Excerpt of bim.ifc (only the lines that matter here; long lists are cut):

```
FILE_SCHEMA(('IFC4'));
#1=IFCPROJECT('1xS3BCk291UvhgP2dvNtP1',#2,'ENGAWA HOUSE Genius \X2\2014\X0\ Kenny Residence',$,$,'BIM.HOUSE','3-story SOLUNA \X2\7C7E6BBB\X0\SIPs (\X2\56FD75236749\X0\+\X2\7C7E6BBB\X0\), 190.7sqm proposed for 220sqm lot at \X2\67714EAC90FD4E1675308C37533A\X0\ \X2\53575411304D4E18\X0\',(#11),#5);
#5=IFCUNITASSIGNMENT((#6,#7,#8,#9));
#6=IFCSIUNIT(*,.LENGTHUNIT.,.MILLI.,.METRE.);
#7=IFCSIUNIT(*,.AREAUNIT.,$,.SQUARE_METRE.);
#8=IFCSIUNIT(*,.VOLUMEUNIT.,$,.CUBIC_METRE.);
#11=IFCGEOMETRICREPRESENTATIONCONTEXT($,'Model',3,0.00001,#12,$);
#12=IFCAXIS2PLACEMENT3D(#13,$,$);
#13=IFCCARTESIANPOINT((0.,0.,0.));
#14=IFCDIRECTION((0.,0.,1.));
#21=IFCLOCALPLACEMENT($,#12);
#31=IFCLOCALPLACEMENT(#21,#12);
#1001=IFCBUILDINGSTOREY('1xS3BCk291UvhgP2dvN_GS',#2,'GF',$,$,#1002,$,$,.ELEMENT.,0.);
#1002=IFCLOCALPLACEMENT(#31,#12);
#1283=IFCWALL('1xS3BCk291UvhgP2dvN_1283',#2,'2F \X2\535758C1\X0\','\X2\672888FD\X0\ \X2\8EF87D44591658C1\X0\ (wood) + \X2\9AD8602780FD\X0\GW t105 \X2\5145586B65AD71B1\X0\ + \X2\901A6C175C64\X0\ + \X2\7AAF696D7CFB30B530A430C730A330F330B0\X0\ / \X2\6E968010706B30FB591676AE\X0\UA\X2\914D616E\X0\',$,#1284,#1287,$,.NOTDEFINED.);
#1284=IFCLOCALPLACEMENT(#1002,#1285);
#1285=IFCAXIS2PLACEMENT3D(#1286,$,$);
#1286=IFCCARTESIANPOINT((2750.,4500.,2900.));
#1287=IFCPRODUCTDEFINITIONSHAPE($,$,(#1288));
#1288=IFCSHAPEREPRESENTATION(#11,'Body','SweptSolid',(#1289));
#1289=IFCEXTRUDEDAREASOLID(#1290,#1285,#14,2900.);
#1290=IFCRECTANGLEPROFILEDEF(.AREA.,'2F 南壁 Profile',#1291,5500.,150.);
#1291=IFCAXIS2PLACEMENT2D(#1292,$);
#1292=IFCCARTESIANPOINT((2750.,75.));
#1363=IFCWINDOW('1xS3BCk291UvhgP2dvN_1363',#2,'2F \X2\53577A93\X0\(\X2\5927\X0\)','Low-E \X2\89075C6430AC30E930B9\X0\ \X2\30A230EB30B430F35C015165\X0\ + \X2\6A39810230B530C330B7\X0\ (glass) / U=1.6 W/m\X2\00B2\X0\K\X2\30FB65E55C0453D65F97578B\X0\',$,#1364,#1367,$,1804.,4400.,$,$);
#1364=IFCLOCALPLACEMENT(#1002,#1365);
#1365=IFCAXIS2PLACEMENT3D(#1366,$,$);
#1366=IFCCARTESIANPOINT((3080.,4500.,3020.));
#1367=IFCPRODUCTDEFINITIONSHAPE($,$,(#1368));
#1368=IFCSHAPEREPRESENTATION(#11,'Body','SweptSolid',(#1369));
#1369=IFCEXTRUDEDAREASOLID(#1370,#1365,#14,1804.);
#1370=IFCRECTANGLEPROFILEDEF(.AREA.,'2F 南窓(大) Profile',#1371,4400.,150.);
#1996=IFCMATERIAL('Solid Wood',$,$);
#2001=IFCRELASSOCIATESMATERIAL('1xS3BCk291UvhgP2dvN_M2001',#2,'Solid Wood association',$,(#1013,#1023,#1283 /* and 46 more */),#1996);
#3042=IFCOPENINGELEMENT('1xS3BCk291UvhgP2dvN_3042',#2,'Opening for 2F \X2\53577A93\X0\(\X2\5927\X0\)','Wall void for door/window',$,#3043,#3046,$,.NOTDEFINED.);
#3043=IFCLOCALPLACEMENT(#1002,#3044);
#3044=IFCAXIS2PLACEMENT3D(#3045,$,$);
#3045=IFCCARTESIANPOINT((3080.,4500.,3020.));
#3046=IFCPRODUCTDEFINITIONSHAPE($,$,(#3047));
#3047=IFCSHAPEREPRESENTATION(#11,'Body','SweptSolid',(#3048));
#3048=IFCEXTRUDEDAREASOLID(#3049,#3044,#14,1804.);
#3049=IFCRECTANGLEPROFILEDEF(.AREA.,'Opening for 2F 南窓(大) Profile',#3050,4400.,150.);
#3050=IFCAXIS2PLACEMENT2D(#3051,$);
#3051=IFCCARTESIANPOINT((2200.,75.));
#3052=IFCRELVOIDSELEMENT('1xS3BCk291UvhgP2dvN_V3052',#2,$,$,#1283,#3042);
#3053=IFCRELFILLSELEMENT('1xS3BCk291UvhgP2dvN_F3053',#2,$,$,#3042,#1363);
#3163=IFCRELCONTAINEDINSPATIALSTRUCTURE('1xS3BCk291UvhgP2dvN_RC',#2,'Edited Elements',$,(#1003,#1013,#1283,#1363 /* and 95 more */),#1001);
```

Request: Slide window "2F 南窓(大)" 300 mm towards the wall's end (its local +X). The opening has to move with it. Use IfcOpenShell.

```python
import ifcopenshell
import ifcopenshell.api.geometry
import ifcopenshell.util.placement
import ifcopenshell.util.unit

model = ifcopenshell.open("bim.ifc")
unit_scale = ifcopenshell.util.unit.calculate_unit_scale(model)

window = model.by_guid("1xS3BCk291UvhgP2dvN_1363")
opening = window.FillsVoids[0].RelatingOpeningElement
wall = opening.VoidsElements[0].RelatingBuildingElement

wall_matrix = ifcopenshell.util.placement.get_local_placement(wall.ObjectPlacement)
shift = wall_matrix[:3, 0] * 0.3 / unit_scale
before = ifcopenshell.util.placement.get_local_placement(window.ObjectPlacement)[:3, 3].copy()

# The window is not placed relative to its opening, so move both.
for product in (opening, window):
    matrix = ifcopenshell.util.placement.get_local_placement(product.ObjectPlacement)
    matrix[:3, 3] += shift
    ifcopenshell.api.geometry.edit_object_placement(model, product=product, matrix=matrix, is_si=False)

after = ifcopenshell.util.placement.get_local_placement(window.ObjectPlacement)[:3, 3]
print("window moved by", (after - before).round(3) + 0.0)

model.write("bim_updated.ifc")
```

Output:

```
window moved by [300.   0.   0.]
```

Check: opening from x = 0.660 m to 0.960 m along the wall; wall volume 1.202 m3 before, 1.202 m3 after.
